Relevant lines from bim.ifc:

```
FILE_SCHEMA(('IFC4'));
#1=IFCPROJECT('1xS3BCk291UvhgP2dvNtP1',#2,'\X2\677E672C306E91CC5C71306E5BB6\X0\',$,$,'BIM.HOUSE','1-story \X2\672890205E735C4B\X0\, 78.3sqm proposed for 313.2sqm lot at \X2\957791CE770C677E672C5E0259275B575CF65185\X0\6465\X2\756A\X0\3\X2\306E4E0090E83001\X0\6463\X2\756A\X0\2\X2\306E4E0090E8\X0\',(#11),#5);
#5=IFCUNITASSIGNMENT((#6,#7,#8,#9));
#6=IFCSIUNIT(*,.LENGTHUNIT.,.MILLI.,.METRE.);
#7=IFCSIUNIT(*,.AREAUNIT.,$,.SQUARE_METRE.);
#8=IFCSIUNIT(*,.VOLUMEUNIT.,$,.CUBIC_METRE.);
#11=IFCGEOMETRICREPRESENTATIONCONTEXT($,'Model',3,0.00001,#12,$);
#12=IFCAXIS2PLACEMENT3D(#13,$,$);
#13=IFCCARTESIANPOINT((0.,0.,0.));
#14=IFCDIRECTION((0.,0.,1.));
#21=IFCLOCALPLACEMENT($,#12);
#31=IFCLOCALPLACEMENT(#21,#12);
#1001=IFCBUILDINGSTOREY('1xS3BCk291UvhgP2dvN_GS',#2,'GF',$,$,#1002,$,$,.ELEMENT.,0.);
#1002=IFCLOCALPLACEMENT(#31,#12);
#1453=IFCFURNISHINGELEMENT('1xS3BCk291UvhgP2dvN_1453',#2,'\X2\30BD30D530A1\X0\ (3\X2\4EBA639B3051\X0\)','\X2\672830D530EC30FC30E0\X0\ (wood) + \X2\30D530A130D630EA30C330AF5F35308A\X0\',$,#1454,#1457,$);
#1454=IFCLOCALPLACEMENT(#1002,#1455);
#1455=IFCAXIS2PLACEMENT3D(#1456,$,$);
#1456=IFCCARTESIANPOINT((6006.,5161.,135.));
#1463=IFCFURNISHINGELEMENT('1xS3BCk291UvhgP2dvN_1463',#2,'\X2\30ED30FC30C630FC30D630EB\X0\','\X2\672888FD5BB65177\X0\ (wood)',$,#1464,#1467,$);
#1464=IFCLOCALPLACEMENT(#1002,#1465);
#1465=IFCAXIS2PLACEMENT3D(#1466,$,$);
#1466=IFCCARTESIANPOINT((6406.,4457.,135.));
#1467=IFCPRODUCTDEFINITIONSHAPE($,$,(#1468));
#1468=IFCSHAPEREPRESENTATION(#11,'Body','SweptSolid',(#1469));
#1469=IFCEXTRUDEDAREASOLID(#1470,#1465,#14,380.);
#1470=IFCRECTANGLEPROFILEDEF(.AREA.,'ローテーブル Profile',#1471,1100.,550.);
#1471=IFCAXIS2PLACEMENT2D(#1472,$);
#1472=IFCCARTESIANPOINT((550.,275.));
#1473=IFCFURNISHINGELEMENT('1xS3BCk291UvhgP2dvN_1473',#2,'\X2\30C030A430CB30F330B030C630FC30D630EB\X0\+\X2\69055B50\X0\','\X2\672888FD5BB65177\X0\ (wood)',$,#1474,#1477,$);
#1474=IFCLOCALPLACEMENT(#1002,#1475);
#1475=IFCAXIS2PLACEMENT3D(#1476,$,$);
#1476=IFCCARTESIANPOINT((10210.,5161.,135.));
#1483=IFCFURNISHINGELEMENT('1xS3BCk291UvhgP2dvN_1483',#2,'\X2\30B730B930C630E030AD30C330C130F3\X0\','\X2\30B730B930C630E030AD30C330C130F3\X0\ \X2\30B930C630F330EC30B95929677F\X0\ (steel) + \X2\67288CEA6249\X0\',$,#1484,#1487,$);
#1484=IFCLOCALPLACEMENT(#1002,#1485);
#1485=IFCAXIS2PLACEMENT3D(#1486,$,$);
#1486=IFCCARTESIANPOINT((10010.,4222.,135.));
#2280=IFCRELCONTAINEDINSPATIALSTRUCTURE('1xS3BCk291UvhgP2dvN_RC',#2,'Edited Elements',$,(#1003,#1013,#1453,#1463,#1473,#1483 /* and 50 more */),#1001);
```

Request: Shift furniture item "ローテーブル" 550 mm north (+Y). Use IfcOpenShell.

```python
import ifcopenshell
import ifcopenshell.api.geometry
import ifcopenshell.util.placement

model = ifcopenshell.open("bim.ifc")

item = model.by_guid("1xS3BCk291UvhgP2dvN_1463")
matrix = ifcopenshell.util.placement.get_local_placement(item.ObjectPlacement)
matrix[1, 3] += 550.0
ifcopenshell.api.geometry.edit_object_placement(model, product=item, matrix=matrix, is_si=False)

print(ifcopenshell.util.placement.get_local_placement(item.ObjectPlacement).round(3) + 0.0)

model.write("bim-out.ifc")
```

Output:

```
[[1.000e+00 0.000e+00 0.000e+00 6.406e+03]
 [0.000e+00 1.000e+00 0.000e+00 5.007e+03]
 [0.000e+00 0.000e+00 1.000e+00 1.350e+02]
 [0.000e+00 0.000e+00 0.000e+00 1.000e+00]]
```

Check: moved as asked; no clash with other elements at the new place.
